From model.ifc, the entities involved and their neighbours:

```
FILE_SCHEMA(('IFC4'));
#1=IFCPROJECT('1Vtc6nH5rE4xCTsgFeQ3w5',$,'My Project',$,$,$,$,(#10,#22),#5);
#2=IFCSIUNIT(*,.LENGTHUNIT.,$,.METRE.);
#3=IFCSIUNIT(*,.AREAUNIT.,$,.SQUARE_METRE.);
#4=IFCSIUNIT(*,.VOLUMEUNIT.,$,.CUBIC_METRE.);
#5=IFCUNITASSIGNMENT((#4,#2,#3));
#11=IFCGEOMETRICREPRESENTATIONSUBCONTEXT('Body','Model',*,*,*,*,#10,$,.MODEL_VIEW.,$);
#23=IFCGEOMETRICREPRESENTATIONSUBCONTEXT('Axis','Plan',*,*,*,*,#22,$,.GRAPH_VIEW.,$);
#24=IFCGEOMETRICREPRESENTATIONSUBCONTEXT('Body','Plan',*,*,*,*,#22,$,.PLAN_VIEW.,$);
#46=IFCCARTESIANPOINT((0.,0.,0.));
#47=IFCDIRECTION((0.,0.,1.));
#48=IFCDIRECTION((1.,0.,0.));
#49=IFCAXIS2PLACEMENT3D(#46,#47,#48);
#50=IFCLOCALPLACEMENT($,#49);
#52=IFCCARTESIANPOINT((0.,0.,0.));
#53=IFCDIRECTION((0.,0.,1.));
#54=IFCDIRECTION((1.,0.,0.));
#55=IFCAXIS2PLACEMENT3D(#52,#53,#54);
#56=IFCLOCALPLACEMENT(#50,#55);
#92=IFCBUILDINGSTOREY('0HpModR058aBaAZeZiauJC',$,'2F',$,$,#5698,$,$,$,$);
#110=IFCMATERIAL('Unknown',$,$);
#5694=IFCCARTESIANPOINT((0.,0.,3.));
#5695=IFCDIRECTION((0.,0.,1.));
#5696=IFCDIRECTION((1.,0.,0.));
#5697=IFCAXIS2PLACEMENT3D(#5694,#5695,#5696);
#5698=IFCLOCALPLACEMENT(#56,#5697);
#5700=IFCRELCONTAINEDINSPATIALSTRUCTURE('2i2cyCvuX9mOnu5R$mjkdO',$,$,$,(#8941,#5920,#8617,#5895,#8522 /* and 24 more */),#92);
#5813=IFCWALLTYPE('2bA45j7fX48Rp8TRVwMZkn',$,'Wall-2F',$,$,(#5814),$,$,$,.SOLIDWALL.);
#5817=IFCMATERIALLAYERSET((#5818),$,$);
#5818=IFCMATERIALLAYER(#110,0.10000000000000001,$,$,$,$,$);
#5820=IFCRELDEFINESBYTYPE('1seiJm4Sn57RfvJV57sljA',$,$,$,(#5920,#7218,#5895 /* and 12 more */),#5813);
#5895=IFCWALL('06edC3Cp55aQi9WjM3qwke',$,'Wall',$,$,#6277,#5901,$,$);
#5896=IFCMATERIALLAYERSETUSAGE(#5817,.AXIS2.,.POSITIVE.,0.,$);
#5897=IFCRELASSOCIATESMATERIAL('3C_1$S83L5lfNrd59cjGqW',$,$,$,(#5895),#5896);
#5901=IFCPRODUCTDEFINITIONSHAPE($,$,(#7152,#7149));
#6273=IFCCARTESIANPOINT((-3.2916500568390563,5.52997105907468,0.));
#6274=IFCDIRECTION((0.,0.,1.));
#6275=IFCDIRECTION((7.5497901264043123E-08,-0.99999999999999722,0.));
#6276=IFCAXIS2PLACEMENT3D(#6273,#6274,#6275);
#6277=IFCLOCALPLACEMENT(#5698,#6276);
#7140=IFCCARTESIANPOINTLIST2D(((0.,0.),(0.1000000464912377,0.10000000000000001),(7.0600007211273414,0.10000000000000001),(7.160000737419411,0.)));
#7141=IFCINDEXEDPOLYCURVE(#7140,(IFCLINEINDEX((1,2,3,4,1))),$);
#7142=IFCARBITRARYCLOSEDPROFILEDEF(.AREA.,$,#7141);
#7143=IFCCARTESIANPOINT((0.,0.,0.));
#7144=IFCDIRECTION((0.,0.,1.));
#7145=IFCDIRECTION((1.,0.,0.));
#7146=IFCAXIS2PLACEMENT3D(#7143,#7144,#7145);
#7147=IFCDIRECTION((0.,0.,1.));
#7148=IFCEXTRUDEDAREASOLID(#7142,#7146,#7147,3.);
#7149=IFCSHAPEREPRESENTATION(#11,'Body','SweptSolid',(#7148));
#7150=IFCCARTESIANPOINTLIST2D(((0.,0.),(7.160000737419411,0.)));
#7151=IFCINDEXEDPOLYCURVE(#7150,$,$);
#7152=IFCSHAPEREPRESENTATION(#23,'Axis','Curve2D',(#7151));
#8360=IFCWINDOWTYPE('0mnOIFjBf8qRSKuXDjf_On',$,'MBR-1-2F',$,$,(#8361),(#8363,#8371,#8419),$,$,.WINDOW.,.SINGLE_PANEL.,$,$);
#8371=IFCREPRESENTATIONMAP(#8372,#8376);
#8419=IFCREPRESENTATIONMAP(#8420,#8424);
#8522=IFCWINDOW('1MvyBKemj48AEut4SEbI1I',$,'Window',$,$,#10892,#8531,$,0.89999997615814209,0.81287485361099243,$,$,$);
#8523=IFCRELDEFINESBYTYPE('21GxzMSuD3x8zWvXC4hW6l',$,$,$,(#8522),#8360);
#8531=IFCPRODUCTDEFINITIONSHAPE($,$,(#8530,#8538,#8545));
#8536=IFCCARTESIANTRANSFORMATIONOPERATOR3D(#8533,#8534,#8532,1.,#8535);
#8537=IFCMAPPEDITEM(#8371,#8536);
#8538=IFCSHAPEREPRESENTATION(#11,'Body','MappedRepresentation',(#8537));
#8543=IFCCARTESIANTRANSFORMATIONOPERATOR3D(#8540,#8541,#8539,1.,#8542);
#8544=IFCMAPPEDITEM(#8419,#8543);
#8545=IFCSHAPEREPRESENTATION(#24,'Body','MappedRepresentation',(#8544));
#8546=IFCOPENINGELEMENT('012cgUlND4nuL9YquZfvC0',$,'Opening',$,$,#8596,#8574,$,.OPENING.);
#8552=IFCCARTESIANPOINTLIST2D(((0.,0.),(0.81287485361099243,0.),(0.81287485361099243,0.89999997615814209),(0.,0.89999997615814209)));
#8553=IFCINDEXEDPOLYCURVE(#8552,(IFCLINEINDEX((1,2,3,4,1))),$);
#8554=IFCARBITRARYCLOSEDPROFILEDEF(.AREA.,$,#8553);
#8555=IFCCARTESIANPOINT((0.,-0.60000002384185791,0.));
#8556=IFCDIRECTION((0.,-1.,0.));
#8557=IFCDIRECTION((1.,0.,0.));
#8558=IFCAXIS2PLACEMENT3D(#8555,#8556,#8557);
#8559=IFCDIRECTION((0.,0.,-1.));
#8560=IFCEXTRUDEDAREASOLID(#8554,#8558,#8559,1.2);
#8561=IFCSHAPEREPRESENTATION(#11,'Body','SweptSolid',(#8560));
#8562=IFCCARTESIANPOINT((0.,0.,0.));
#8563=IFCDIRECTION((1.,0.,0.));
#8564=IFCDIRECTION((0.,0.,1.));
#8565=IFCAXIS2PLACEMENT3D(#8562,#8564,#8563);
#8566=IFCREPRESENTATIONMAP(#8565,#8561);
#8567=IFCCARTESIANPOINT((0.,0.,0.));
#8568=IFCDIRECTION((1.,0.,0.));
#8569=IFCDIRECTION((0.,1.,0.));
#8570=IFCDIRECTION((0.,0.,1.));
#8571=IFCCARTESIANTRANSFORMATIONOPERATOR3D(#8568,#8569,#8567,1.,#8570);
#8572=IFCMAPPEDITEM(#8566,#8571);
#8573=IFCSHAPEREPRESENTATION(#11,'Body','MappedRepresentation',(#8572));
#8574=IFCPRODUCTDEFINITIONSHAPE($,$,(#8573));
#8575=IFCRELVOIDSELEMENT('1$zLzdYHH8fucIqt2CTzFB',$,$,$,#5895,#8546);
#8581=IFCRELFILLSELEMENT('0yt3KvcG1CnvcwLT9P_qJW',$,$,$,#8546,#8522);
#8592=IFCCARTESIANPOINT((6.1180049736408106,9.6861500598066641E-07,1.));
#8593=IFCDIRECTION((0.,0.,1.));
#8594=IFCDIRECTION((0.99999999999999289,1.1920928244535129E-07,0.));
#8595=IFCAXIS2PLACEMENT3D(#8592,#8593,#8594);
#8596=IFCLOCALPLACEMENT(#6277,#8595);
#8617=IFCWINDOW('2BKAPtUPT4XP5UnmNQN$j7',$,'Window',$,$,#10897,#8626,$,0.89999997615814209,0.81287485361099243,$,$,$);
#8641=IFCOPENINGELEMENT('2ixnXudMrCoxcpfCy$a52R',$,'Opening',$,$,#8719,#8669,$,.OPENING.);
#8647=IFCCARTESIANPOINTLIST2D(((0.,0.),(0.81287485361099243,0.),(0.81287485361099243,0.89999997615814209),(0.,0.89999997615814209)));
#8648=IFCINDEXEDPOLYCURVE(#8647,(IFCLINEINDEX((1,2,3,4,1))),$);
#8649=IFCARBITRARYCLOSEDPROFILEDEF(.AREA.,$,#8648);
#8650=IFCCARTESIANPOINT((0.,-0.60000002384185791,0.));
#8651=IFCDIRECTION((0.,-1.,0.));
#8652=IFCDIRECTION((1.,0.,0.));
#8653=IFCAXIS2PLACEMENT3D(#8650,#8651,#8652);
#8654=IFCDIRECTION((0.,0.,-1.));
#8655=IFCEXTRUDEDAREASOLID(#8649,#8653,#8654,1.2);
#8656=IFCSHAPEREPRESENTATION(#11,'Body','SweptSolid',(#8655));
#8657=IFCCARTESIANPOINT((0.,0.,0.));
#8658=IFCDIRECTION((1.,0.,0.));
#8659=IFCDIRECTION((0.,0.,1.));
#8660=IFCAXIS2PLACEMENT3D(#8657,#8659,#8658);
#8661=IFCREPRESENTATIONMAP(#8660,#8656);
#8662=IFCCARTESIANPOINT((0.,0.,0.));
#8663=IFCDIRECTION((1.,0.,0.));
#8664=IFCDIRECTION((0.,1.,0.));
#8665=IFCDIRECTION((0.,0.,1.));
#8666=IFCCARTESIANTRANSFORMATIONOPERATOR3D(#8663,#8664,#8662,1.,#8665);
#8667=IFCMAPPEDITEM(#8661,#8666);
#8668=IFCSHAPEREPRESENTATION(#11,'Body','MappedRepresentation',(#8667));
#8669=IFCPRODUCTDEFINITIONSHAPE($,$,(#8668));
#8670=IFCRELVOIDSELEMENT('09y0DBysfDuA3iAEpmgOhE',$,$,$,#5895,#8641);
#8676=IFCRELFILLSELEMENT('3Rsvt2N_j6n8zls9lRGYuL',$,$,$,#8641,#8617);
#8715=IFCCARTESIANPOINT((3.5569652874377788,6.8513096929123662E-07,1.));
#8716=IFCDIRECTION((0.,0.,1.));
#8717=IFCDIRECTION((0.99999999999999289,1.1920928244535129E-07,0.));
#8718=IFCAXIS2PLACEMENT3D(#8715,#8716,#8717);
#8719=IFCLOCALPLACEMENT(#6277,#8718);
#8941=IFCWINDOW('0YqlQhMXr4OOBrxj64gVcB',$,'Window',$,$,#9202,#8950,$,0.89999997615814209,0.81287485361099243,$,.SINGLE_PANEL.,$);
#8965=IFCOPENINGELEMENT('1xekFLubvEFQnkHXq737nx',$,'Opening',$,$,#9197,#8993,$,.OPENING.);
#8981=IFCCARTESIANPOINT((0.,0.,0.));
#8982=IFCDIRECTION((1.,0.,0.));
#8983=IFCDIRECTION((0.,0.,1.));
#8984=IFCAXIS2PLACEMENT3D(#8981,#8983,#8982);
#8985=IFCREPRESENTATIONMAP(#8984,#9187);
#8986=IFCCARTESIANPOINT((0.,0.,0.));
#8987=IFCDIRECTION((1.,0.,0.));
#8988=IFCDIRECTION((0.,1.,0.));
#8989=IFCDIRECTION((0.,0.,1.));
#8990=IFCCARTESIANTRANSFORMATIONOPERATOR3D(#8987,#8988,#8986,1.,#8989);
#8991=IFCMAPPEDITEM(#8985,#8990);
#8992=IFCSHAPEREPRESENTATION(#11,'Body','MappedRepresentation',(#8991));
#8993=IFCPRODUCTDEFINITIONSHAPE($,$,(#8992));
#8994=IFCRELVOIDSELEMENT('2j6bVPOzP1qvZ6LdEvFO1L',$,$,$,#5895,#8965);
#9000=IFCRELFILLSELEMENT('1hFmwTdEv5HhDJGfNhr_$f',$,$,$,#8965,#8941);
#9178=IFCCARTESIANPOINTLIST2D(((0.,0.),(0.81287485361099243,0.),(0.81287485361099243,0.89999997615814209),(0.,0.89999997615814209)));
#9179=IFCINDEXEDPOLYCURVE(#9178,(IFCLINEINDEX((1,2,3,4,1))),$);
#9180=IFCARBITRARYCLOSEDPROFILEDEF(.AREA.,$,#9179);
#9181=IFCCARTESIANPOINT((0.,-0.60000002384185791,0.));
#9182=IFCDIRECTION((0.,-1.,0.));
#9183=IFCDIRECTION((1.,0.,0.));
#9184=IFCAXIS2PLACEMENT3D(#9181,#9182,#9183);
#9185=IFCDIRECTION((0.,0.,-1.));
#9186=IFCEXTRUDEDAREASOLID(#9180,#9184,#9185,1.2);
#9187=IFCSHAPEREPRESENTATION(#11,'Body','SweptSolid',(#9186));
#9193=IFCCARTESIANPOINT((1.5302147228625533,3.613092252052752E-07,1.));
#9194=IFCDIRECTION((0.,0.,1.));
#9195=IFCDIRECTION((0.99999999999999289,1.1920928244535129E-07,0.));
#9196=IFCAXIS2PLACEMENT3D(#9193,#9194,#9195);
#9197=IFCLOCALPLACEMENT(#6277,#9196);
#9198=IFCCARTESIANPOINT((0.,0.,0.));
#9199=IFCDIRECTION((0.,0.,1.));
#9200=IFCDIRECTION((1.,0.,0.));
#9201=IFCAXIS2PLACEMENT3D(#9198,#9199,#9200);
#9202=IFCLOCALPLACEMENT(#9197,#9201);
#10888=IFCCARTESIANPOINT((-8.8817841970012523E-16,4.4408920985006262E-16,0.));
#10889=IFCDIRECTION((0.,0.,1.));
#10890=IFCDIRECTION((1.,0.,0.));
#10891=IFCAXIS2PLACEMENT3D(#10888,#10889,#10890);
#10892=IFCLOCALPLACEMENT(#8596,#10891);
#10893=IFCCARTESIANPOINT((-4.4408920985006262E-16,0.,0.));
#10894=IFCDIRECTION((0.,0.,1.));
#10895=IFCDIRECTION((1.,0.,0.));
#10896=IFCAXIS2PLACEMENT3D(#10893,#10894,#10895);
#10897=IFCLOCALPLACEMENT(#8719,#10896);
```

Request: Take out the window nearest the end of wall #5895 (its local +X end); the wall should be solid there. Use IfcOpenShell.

```python
import ifcopenshell
import ifcopenshell.api.feature
import ifcopenshell.api.root
import ifcopenshell.geom
import ifcopenshell.util.shape

model = ifcopenshell.open("model.ifc")
settings = ifcopenshell.geom.settings()


def volume(element):
    """Net volume in cubic metres, openings subtracted."""
    shape = ifcopenshell.geom.create_shape(settings, element)
    return ifcopenshell.util.shape.get_volume(shape.geometry)


window = model.by_guid("1MvyBKemj48AEut4SEbI1I")
opening = window.FillsVoids[0].RelatingOpeningElement
wall = opening.VoidsElements[0].RelatingBuildingElement
before = volume(wall)

ifcopenshell.api.root.remove_product(model, product=window)
ifcopenshell.api.feature.remove_feature(model, feature=opening)

after = volume(wall)

print(f"wall volume {before:.3f} -> {after:.3f} m3")

model.write("model_edited.ifc")
```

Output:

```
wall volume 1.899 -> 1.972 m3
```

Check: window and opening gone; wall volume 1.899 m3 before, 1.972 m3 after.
